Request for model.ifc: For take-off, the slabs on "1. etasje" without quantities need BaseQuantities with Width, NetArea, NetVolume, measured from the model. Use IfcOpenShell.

First a look at what the model holds.

```python
import ifcopenshell
import ifcopenshell.util.element
import ifcopenshell.util.unit

model = ifcopenshell.open("model.ifc")
print(model.schema)
for unit_type in ("LENGTHUNIT", "AREAUNIT", "VOLUMEUNIT"):
    print(unit_type, ifcopenshell.util.unit.calculate_unit_scale(model, unit_type))
storey = next(s for s in model.by_type("IfcBuildingStorey") if s.Name == "1. etasje")
slabs = [e for e in ifcopenshell.util.element.get_decomposition(storey) if e.is_a("IfcSlab")]
for e in sorted(slabs, key=lambda e: e.id()):
    print(e.id(), e.is_a(), e.Name, list(ifcopenshell.util.element.get_psets(e, qtos_only=True)), sep=" | ")
```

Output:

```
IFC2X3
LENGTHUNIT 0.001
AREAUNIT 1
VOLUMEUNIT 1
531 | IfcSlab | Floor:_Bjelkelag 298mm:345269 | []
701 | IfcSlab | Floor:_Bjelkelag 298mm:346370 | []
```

```python
import ifcopenshell
import ifcopenshell.api.pset
import ifcopenshell.geom
import ifcopenshell.util.element
import ifcopenshell.util.shape
import ifcopenshell.util.unit

model = ifcopenshell.open("model.ifc")
unit_scale = ifcopenshell.util.unit.calculate_unit_scale(model)
area_scale = ifcopenshell.util.unit.calculate_unit_scale(model, "AREAUNIT")
volume_scale = ifcopenshell.util.unit.calculate_unit_scale(model, "VOLUMEUNIT")
settings = ifcopenshell.geom.settings()

storey = next(s for s in model.by_type("IfcBuildingStorey") if s.Name == "1. etasje")
slabs = [e for e in ifcopenshell.util.element.get_decomposition(storey) if e.is_a("IfcSlab")]

for e in sorted(slabs, key=lambda e: e.id()):
    if ifcopenshell.util.element.get_psets(e, qtos_only=True, should_inherit=False):
        continue
    # Geometry comes back in metres, in the element's own axes.
    shape = ifcopenshell.geom.create_shape(settings, e)
    values = {
        "Width": ifcopenshell.util.shape.get_z(shape.geometry) / unit_scale,
        "NetArea": ifcopenshell.util.shape.get_footprint_area(shape.geometry) / area_scale,
        "NetVolume": ifcopenshell.util.shape.get_volume(shape.geometry) / volume_scale,
    }
    qto = ifcopenshell.api.pset.add_qto(model, product=e, name="BaseQuantities")
    ifcopenshell.api.pset.edit_qto(model, qto=qto, properties=values)
    print(e.id(), {k: round(v, 3) for k, v in values.items()})

model.write("model_v2.ifc")
```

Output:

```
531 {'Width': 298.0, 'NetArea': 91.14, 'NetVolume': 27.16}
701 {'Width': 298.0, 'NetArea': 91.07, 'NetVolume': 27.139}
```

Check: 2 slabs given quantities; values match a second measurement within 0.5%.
